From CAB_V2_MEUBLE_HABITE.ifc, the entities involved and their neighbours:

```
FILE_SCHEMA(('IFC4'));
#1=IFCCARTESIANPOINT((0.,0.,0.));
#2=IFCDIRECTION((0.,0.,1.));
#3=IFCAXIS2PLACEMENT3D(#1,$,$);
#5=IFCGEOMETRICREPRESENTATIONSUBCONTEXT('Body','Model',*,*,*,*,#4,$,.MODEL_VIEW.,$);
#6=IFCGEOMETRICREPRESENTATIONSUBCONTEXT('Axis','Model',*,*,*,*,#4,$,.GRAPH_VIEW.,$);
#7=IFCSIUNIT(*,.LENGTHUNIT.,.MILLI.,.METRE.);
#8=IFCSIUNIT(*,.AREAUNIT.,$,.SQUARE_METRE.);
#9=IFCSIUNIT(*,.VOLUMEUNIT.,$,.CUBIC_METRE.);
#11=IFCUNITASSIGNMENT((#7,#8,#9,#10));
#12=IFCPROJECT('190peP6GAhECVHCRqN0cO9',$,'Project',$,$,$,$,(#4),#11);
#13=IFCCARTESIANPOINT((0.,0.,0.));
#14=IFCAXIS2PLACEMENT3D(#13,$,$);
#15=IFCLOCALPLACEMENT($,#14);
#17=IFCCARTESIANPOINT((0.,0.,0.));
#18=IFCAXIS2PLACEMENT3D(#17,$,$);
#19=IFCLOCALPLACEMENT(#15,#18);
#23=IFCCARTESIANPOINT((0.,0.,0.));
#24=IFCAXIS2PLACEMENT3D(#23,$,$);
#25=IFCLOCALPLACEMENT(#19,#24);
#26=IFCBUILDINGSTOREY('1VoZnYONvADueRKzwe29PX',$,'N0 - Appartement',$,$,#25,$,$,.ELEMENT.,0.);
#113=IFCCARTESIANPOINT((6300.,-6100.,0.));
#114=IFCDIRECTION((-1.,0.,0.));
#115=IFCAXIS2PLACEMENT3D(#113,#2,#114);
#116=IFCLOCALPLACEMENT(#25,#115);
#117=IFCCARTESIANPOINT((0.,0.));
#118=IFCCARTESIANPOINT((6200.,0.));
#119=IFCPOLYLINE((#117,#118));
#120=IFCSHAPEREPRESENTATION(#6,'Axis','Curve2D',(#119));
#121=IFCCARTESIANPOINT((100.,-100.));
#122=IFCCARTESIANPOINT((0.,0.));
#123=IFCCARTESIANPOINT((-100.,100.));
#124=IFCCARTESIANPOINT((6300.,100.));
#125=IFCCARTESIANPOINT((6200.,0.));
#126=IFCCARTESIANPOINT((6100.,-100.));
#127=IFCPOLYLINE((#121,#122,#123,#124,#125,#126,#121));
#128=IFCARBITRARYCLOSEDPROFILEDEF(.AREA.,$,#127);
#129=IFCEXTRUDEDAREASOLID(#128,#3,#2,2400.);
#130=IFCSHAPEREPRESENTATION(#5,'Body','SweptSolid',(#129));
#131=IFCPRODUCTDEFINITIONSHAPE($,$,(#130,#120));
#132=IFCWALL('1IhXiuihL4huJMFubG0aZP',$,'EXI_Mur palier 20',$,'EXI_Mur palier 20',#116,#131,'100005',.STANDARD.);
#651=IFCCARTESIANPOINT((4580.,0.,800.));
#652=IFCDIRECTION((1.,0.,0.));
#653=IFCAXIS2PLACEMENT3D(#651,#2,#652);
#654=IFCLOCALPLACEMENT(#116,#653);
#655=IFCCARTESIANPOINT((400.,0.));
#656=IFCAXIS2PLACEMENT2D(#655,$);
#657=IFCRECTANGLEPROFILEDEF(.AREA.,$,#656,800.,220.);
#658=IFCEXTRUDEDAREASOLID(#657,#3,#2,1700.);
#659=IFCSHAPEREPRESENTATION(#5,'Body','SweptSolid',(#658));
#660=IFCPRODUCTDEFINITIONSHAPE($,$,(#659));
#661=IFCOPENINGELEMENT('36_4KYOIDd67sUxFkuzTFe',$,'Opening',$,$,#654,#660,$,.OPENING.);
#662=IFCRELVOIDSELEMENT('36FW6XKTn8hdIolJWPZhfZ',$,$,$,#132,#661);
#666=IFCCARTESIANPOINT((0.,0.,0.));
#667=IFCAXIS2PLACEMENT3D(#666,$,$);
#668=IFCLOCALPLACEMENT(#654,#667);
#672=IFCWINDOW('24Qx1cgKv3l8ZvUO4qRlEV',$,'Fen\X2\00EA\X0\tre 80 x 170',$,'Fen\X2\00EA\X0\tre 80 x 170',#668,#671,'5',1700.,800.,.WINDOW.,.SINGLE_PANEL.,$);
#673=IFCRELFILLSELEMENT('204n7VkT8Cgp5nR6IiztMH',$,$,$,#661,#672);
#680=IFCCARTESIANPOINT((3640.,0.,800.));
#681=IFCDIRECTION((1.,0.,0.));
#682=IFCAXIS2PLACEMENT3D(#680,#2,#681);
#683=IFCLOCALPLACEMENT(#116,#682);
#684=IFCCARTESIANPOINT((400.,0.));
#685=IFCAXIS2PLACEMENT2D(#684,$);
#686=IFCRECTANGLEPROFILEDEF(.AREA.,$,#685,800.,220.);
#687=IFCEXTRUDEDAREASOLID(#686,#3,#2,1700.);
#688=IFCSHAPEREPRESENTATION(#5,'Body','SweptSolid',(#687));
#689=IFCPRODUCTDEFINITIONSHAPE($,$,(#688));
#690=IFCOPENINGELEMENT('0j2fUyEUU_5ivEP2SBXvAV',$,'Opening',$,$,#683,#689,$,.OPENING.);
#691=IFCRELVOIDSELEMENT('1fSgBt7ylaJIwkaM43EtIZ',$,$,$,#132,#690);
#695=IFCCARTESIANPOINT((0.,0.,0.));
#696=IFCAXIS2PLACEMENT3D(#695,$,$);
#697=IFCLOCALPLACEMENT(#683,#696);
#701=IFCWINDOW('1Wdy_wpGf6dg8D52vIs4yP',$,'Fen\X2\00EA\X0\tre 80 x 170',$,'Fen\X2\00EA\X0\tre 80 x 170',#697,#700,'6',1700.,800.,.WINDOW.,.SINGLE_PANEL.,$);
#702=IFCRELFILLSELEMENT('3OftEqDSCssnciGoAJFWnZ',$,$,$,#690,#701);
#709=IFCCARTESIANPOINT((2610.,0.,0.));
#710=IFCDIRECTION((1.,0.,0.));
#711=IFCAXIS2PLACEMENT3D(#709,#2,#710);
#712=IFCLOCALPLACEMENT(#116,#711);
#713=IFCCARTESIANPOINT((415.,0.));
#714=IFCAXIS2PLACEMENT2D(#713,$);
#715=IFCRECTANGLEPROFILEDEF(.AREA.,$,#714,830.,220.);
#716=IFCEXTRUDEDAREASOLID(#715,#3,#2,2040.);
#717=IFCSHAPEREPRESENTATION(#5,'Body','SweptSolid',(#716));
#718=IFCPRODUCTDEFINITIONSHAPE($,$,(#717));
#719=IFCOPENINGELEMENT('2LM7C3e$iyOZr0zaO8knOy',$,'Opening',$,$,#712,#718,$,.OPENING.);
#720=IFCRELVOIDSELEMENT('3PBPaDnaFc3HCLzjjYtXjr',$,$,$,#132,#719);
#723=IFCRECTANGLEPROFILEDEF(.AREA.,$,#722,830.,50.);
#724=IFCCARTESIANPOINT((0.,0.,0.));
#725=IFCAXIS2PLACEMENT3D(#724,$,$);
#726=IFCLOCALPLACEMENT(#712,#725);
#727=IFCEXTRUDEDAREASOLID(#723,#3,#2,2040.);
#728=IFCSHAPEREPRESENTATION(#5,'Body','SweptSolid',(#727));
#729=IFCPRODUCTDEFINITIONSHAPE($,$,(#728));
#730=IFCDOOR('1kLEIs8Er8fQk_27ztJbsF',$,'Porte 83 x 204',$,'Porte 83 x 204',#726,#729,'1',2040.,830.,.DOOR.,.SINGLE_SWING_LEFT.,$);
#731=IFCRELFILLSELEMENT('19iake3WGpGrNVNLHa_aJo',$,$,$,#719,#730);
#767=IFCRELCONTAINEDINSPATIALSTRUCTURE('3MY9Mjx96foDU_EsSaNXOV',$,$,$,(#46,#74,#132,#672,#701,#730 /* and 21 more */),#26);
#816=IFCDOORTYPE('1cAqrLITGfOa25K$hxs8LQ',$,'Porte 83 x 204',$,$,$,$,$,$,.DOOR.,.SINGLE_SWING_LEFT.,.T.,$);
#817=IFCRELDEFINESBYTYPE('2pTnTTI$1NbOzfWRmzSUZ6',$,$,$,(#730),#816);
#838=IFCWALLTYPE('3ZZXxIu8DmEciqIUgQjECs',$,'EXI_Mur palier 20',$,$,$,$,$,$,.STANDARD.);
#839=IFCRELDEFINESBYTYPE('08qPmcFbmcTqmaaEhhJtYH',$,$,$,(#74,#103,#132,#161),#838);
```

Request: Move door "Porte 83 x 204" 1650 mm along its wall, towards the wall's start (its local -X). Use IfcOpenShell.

```python
import ifcopenshell
import ifcopenshell.api.geometry
import ifcopenshell.util.placement
import ifcopenshell.util.unit

model = ifcopenshell.open("CAB_V2_MEUBLE_HABITE.ifc")
unit_scale = ifcopenshell.util.unit.calculate_unit_scale(model)

door = model.by_guid("1kLEIs8Er8fQk_27ztJbsF")
opening = door.FillsVoids[0].RelatingOpeningElement
wall = opening.VoidsElements[0].RelatingBuildingElement

wall_matrix = ifcopenshell.util.placement.get_local_placement(wall.ObjectPlacement)
shift = wall_matrix[:3, 0] * -1.65 / unit_scale
before = ifcopenshell.util.placement.get_local_placement(door.ObjectPlacement)[:3, 3].copy()

# The door is placed relative to its opening, so it follows when the opening moves.
matrix = ifcopenshell.util.placement.get_local_placement(opening.ObjectPlacement)
matrix[:3, 3] += shift
ifcopenshell.api.geometry.edit_object_placement(
    model, product=opening, matrix=matrix, is_si=False, should_transform_children=True
)

after = ifcopenshell.util.placement.get_local_placement(door.ObjectPlacement)[:3, 3]
print("door moved by", (after - before).round(3) + 0.0)

model.write("CAB_V2_MEUBLE_HABITE_updated.ifc")
```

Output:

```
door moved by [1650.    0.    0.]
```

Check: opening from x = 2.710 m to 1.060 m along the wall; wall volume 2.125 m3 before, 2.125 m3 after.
